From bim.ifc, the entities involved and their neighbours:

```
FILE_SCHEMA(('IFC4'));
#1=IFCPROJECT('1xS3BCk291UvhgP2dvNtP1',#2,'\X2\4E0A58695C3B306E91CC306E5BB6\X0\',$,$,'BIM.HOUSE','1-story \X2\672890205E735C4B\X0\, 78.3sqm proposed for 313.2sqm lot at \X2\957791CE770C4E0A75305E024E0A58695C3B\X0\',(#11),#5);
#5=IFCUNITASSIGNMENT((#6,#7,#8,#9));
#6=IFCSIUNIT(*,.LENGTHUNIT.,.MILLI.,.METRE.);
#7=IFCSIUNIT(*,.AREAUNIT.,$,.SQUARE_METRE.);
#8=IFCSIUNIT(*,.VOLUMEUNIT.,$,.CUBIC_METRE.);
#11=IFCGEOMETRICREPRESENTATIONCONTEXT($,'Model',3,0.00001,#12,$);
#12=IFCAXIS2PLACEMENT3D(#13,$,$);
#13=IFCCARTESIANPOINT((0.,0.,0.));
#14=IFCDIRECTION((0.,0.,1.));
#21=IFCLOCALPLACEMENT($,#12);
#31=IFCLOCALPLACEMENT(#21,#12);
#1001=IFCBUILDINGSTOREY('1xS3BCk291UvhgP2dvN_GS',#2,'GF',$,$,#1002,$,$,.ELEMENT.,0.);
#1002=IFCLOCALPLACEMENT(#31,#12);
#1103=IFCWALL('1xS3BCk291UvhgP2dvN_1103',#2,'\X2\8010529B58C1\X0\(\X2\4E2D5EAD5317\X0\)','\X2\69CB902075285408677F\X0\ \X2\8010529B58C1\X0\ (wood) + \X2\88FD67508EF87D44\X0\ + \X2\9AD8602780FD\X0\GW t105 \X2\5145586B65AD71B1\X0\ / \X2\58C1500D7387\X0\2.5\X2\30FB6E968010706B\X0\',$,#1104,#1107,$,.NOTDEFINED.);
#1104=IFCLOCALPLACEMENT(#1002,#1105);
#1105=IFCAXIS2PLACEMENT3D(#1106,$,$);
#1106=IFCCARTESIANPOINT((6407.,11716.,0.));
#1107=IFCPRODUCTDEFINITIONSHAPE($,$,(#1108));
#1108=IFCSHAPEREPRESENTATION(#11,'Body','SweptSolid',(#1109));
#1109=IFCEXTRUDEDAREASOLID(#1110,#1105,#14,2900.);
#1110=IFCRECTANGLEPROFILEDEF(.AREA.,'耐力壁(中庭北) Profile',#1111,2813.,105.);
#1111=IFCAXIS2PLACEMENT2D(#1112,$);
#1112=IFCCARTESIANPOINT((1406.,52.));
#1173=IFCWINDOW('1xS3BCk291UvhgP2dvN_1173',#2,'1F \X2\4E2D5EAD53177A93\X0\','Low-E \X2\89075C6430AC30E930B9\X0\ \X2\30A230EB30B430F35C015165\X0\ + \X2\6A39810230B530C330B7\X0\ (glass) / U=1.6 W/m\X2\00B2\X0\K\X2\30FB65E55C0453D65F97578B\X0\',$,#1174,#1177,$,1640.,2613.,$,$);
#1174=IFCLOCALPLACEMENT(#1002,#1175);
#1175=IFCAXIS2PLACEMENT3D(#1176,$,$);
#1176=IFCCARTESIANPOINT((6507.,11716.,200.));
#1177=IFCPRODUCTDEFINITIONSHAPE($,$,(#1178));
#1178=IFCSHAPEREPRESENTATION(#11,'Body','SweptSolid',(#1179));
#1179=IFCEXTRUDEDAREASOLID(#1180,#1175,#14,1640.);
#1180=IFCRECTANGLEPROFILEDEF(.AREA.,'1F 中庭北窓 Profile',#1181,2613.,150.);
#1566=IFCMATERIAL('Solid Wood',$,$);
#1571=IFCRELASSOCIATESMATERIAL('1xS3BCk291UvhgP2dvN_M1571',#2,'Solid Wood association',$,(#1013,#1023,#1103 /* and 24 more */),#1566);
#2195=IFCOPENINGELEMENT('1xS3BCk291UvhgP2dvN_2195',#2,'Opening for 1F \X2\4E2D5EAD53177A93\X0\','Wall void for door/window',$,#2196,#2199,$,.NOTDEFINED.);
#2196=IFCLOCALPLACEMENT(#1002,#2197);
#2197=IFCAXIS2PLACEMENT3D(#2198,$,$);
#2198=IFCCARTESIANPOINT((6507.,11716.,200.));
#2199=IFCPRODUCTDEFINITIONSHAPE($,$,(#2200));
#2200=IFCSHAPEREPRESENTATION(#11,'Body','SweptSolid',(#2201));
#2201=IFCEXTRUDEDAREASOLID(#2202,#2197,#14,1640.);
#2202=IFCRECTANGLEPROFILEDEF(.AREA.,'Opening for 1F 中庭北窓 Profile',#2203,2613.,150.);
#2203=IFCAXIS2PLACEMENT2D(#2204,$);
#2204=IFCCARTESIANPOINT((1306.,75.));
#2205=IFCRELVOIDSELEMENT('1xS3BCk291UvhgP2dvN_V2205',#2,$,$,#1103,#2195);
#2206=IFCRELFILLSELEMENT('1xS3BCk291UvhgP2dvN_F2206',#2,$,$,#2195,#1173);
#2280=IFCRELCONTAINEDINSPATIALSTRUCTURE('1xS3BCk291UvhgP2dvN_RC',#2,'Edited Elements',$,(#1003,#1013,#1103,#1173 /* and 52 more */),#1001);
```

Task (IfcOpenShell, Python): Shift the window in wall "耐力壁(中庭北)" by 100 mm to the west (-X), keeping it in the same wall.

```python
import ifcopenshell
import ifcopenshell.api.geometry
import ifcopenshell.util.placement
import ifcopenshell.util.unit

model = ifcopenshell.open("bim.ifc")
unit_scale = ifcopenshell.util.unit.calculate_unit_scale(model)

window = model.by_guid("1xS3BCk291UvhgP2dvN_1173")
opening = window.FillsVoids[0].RelatingOpeningElement
wall = opening.VoidsElements[0].RelatingBuildingElement

wall_matrix = ifcopenshell.util.placement.get_local_placement(wall.ObjectPlacement)
shift = wall_matrix[:3, 0] * -0.1 / unit_scale
before = ifcopenshell.util.placement.get_local_placement(window.ObjectPlacement)[:3, 3].copy()

# The window is not placed relative to its opening, so move both.
for product in (opening, window):
    matrix = ifcopenshell.util.placement.get_local_placement(product.ObjectPlacement)
    matrix[:3, 3] += shift
    ifcopenshell.api.geometry.edit_object_placement(model, product=product, matrix=matrix, is_si=False)

after = ifcopenshell.util.placement.get_local_placement(window.ObjectPlacement)[:3, 3]
print("window moved by", (after - before).round(3) + 0.0)

model.write("bim_edited.ifc")
```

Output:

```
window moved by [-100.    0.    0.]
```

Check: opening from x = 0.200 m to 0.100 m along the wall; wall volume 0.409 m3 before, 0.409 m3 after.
